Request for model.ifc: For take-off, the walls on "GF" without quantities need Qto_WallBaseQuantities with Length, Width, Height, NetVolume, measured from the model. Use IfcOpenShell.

First a look at what the model holds.

```python
import ifcopenshell
import ifcopenshell.util.element
import ifcopenshell.util.unit

model = ifcopenshell.open("model.ifc")
print(model.schema)
for unit_type in ("LENGTHUNIT", "AREAUNIT", "VOLUMEUNIT"):
    print(unit_type, ifcopenshell.util.unit.calculate_unit_scale(model, unit_type))
storey = next(s for s in model.by_type("IfcBuildingStorey") if s.Name == "GF")
walls = [e for e in ifcopenshell.util.element.get_decomposition(storey) if e.is_a("IfcWall")]
for e in sorted(walls, key=lambda e: e.id()):
    print(e.id(), e.is_a(), e.Name, list(ifcopenshell.util.element.get_psets(e, qtos_only=True)), sep=" | ")
```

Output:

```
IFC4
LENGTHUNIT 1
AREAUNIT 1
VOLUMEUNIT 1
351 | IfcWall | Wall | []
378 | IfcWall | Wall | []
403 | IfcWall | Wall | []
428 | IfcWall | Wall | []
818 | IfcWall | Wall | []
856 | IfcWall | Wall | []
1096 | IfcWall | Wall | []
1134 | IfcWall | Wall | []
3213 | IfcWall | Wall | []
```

```python
import ifcopenshell
import ifcopenshell.api.pset
import ifcopenshell.geom
import ifcopenshell.util.element
import ifcopenshell.util.shape
import ifcopenshell.util.unit

model = ifcopenshell.open("model.ifc")
unit_scale = ifcopenshell.util.unit.calculate_unit_scale(model)
volume_scale = ifcopenshell.util.unit.calculate_unit_scale(model, "VOLUMEUNIT")
settings = ifcopenshell.geom.settings()

storey = next(s for s in model.by_type("IfcBuildingStorey") if s.Name == "GF")
walls = [e for e in ifcopenshell.util.element.get_decomposition(storey) if e.is_a("IfcWall")]

for e in sorted(walls, key=lambda e: e.id()):
    if ifcopenshell.util.element.get_psets(e, qtos_only=True, should_inherit=False):
        continue
    # Geometry comes back in metres, in the element's own axes.
    shape = ifcopenshell.geom.create_shape(settings, e)
    values = {
        "Length": ifcopenshell.util.shape.get_x(shape.geometry) / unit_scale,
        "Width": ifcopenshell.util.shape.get_y(shape.geometry) / unit_scale,
        "Height": ifcopenshell.util.shape.get_z(shape.geometry) / unit_scale,
        "NetVolume": ifcopenshell.util.shape.get_volume(shape.geometry) / volume_scale,
    }
    qto = ifcopenshell.api.pset.add_qto(model, product=e, name="Qto_WallBaseQuantities")
    ifcopenshell.api.pset.edit_qto(model, qto=qto, properties=values)
    print(e.id(), {k: round(v, 3) for k, v in values.items()})

model.write("model_rev.ifc")
```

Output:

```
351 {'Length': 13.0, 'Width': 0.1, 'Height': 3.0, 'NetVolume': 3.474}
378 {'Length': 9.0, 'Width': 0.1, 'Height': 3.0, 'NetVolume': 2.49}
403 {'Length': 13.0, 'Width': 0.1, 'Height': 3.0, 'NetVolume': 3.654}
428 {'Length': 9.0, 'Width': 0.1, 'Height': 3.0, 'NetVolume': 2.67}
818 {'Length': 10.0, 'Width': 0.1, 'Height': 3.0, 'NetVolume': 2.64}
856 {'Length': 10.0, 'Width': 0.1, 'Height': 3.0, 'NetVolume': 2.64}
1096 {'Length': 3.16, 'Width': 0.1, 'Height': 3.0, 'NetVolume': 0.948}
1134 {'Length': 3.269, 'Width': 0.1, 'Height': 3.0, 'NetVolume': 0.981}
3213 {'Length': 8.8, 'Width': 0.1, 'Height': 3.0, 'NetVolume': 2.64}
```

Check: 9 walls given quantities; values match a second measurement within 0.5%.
